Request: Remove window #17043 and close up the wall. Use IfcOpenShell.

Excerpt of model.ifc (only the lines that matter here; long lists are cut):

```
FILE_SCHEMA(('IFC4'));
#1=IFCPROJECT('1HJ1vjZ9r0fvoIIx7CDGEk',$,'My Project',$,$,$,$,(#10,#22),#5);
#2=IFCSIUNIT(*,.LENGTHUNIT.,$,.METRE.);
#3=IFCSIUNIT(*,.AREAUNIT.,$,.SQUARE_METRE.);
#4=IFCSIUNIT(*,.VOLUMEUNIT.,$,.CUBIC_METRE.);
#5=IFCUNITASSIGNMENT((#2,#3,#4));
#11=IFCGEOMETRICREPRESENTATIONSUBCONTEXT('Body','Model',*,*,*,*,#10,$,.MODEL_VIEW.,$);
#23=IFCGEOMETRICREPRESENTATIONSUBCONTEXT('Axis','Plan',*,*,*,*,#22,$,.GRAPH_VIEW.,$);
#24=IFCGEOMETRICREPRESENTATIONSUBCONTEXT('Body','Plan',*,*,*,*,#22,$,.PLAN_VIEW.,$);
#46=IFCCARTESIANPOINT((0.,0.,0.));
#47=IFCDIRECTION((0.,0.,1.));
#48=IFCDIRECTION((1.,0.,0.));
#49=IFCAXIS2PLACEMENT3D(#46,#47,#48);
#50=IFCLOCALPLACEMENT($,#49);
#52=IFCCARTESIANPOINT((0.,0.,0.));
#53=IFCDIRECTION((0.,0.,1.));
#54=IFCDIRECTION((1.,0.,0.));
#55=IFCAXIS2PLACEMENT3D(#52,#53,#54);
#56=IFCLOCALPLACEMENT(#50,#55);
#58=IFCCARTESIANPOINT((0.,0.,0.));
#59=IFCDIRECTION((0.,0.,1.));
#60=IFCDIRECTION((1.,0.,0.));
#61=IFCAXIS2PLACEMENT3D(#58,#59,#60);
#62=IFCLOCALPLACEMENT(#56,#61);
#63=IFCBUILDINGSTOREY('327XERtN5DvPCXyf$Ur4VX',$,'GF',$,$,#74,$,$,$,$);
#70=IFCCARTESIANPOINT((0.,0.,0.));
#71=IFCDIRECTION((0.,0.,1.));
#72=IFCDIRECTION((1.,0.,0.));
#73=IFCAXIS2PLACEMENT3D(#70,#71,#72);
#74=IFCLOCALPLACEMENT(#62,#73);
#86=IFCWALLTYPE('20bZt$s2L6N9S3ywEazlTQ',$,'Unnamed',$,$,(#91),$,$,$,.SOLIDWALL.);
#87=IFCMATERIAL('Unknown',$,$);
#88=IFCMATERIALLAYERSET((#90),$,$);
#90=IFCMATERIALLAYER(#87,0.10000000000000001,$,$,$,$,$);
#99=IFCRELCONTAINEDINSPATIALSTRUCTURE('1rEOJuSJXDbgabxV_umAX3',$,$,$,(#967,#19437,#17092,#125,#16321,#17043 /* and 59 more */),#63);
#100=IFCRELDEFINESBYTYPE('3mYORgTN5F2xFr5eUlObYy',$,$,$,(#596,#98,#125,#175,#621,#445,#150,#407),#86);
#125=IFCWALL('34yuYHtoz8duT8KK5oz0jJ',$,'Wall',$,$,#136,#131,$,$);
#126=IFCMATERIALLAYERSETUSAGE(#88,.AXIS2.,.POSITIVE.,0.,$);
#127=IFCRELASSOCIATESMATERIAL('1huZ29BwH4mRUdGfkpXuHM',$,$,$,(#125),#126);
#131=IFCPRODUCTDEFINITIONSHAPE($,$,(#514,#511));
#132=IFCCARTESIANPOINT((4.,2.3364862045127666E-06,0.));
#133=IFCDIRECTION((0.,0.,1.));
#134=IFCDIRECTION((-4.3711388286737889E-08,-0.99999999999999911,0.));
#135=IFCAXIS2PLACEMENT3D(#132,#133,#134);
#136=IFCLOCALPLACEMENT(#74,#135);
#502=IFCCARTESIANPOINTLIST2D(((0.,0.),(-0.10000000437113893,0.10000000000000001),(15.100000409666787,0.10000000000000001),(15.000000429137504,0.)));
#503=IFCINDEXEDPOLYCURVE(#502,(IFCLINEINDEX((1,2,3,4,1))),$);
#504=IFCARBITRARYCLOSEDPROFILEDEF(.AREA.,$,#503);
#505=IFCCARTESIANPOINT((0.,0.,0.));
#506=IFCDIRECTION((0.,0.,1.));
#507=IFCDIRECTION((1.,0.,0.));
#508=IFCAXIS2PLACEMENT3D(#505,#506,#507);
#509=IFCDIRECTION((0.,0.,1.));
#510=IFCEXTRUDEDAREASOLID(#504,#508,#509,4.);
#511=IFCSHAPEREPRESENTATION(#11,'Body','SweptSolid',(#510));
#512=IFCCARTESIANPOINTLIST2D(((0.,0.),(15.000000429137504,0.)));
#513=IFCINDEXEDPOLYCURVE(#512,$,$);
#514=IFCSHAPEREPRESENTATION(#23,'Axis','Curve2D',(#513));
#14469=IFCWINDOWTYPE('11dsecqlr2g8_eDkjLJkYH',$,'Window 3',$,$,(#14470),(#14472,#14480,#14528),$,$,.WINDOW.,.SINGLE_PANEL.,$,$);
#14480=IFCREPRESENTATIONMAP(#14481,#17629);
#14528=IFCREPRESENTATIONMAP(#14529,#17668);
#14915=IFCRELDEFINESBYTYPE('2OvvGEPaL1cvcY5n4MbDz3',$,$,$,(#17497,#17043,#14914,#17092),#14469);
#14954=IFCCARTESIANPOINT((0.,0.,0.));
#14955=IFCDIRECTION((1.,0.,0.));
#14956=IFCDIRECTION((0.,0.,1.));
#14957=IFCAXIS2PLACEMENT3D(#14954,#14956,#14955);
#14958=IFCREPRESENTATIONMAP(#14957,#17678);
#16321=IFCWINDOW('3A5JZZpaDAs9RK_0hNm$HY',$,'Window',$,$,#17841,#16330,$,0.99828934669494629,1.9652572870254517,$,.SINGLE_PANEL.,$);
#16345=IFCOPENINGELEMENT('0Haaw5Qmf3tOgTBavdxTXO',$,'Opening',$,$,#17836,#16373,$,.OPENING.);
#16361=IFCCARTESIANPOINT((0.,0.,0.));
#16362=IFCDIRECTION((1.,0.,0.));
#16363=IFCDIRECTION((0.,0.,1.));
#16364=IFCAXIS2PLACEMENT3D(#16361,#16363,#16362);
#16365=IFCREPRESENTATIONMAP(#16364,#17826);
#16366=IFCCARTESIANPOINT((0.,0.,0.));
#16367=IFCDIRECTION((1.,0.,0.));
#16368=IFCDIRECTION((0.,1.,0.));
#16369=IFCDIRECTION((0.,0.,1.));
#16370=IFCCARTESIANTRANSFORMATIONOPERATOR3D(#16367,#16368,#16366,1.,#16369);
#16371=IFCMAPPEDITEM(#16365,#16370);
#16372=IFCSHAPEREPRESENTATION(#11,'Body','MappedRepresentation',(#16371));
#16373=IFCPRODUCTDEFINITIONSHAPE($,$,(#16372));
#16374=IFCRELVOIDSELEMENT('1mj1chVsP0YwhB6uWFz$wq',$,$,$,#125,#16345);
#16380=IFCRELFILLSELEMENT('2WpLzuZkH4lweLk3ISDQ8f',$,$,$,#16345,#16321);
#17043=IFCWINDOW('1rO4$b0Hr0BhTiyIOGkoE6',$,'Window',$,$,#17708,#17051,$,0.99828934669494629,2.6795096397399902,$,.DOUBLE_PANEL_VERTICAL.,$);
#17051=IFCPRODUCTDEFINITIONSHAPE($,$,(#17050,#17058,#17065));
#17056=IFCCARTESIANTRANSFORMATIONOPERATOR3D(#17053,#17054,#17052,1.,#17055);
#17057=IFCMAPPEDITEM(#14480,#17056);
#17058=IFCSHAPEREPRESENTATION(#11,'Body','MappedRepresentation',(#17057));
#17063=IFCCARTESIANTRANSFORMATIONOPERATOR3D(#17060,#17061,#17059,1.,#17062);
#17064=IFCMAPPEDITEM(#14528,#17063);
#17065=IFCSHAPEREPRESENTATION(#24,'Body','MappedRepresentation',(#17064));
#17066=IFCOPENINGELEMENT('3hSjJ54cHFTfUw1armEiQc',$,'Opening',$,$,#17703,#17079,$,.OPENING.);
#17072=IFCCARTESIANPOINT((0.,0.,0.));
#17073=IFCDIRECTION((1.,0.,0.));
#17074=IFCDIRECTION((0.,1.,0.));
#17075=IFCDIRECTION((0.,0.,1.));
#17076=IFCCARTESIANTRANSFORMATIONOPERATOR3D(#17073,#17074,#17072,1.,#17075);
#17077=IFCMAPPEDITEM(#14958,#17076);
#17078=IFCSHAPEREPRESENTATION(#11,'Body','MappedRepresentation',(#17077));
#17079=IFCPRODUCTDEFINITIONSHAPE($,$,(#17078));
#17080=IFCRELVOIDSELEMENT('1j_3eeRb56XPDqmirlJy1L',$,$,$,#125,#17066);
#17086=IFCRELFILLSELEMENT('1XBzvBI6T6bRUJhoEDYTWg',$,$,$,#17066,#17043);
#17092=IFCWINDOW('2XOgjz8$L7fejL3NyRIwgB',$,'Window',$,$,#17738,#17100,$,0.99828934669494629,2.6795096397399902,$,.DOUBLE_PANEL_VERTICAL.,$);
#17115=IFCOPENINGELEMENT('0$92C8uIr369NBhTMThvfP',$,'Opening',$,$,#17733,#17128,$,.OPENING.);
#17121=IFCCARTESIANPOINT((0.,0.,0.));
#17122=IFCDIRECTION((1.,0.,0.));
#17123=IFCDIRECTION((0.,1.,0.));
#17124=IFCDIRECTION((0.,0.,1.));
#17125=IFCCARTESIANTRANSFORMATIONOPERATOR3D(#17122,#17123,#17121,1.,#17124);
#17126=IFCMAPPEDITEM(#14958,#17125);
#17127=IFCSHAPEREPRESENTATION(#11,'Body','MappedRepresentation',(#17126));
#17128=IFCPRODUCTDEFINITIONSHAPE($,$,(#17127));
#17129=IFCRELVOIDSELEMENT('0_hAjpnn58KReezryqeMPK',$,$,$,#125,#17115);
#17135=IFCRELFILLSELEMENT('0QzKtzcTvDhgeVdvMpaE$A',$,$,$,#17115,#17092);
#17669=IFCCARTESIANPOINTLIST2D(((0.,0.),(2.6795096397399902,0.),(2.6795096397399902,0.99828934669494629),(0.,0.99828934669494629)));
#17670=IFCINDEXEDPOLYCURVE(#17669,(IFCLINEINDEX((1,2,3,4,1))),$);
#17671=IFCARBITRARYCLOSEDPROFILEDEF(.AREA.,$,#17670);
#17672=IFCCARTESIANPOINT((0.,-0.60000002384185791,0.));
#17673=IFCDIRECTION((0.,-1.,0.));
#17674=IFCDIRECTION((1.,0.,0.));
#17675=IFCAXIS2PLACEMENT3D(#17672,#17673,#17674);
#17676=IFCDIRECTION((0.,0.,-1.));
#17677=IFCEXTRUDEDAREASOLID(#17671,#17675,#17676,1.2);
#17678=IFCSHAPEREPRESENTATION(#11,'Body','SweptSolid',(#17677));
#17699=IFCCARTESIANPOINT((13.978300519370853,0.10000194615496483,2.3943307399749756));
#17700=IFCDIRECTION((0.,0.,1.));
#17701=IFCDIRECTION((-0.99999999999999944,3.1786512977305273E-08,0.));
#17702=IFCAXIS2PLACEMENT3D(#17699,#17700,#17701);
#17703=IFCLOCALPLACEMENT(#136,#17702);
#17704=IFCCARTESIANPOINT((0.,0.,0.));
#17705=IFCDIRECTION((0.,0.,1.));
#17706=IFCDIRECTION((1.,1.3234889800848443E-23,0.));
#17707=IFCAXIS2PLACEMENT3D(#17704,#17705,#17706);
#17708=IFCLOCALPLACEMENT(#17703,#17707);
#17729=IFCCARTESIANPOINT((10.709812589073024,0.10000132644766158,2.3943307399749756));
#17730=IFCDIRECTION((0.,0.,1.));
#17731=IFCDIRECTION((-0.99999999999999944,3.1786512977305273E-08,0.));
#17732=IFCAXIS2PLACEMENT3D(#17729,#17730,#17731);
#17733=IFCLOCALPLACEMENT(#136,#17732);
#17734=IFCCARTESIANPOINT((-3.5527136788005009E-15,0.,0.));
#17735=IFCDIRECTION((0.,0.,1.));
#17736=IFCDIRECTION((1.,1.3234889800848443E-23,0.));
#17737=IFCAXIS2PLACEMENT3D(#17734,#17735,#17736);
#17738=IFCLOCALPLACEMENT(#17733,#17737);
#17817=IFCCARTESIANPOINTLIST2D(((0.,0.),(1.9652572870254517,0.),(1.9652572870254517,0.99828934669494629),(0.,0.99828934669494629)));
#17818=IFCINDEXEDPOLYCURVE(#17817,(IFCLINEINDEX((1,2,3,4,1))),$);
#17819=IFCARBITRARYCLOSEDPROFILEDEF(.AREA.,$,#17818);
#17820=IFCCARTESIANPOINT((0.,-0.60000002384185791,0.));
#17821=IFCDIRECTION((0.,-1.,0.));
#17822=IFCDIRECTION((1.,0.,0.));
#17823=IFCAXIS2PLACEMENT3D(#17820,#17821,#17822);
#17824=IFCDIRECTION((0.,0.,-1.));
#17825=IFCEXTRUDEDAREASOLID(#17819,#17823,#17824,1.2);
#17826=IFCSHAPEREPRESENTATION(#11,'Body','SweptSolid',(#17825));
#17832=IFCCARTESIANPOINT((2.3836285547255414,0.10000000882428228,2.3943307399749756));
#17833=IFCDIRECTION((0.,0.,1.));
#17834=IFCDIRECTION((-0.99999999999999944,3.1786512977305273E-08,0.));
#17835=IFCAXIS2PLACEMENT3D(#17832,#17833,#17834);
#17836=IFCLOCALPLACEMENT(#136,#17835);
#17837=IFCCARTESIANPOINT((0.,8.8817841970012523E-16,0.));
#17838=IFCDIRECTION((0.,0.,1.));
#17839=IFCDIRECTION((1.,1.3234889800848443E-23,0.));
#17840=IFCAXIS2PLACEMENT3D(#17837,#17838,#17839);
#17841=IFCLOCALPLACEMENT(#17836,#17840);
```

```python
import ifcopenshell
import ifcopenshell.api.feature
import ifcopenshell.api.root
import ifcopenshell.geom
import ifcopenshell.util.shape

model = ifcopenshell.open("model.ifc")
settings = ifcopenshell.geom.settings()


def volume(element):
    """Net volume in cubic metres, openings subtracted."""
    shape = ifcopenshell.geom.create_shape(settings, element)
    return ifcopenshell.util.shape.get_volume(shape.geometry)


window = model.by_id(17043)
opening = window.FillsVoids[0].RelatingOpeningElement
wall = opening.VoidsElements[0].RelatingBuildingElement
before = volume(wall)

ifcopenshell.api.root.remove_product(model, product=window)
ifcopenshell.api.feature.remove_feature(model, feature=opening)

after = volume(wall)

print(f"wall volume {before:.3f} -> {after:.3f} m3")

model.write("model_edited.ifc")
```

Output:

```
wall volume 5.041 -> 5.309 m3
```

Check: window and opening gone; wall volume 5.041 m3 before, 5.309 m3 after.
